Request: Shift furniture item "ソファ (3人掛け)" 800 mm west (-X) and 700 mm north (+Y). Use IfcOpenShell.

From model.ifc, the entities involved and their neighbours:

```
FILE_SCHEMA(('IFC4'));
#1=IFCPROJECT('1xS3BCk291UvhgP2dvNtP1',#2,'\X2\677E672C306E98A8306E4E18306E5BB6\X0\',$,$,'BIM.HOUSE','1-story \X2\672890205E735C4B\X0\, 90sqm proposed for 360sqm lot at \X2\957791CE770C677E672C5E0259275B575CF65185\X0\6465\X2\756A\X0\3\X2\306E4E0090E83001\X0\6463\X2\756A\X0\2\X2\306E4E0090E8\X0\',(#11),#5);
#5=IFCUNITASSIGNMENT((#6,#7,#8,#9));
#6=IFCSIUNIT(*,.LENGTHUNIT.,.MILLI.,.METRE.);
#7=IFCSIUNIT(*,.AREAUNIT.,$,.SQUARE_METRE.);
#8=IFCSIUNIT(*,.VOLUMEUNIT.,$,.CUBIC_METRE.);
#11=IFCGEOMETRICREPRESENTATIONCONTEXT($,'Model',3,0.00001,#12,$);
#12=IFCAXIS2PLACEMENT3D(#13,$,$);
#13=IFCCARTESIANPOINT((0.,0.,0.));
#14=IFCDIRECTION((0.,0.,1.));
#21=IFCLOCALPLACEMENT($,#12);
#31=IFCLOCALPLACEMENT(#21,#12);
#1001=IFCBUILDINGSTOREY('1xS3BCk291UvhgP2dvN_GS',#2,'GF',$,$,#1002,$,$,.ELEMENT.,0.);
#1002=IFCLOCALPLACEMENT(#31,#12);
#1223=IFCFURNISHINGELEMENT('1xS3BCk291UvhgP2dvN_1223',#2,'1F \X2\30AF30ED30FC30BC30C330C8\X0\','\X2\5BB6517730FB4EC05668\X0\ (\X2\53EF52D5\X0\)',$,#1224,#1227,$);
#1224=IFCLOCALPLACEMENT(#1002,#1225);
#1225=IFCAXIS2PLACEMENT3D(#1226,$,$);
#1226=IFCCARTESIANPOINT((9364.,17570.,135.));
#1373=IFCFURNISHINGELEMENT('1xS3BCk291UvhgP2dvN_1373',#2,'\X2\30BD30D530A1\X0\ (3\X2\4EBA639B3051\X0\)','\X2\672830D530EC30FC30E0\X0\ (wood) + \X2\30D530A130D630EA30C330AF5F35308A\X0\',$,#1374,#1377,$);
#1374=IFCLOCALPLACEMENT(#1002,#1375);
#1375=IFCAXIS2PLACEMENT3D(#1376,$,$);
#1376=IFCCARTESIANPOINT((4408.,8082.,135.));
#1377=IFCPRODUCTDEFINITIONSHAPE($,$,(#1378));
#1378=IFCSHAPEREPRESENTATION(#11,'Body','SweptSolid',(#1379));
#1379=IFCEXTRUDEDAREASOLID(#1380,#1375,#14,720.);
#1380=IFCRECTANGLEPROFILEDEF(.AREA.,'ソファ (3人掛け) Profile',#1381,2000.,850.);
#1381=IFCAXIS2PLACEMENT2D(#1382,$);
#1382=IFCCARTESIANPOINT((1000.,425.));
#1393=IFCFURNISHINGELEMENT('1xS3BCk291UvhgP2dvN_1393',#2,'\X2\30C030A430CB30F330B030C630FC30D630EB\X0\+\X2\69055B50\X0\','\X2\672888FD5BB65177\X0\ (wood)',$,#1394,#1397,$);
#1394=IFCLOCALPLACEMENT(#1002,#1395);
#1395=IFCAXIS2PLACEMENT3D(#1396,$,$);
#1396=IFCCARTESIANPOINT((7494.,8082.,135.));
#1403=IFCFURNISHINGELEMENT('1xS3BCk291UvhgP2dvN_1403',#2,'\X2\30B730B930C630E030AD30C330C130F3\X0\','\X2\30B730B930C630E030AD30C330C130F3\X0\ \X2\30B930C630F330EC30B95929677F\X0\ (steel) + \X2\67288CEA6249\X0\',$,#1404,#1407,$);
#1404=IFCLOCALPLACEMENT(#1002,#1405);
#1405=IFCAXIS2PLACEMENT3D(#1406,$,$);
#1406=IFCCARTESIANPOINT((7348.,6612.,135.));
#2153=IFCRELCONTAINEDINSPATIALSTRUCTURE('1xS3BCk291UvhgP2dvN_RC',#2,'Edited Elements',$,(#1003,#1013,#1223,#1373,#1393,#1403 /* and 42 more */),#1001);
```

```python
import ifcopenshell
import ifcopenshell.api.geometry
import ifcopenshell.util.placement
import ifcopenshell.util.unit

model = ifcopenshell.open("model.ifc")
unit_scale = ifcopenshell.util.unit.calculate_unit_scale(model)

item = model.by_guid("1xS3BCk291UvhgP2dvN_1373")
matrix = ifcopenshell.util.placement.get_local_placement(item.ObjectPlacement)
matrix[0, 3] -= 0.8 / unit_scale
matrix[1, 3] += 0.7 / unit_scale
ifcopenshell.api.geometry.edit_object_placement(model, product=item, matrix=matrix, is_si=False)

print(ifcopenshell.util.placement.get_local_placement(item.ObjectPlacement).round(3) + 0.0)

model.write("model_v2.ifc")
```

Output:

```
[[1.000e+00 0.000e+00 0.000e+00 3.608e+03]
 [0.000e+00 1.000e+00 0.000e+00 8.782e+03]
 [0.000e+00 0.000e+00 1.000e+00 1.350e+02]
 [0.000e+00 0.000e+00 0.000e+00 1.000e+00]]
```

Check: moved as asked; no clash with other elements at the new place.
